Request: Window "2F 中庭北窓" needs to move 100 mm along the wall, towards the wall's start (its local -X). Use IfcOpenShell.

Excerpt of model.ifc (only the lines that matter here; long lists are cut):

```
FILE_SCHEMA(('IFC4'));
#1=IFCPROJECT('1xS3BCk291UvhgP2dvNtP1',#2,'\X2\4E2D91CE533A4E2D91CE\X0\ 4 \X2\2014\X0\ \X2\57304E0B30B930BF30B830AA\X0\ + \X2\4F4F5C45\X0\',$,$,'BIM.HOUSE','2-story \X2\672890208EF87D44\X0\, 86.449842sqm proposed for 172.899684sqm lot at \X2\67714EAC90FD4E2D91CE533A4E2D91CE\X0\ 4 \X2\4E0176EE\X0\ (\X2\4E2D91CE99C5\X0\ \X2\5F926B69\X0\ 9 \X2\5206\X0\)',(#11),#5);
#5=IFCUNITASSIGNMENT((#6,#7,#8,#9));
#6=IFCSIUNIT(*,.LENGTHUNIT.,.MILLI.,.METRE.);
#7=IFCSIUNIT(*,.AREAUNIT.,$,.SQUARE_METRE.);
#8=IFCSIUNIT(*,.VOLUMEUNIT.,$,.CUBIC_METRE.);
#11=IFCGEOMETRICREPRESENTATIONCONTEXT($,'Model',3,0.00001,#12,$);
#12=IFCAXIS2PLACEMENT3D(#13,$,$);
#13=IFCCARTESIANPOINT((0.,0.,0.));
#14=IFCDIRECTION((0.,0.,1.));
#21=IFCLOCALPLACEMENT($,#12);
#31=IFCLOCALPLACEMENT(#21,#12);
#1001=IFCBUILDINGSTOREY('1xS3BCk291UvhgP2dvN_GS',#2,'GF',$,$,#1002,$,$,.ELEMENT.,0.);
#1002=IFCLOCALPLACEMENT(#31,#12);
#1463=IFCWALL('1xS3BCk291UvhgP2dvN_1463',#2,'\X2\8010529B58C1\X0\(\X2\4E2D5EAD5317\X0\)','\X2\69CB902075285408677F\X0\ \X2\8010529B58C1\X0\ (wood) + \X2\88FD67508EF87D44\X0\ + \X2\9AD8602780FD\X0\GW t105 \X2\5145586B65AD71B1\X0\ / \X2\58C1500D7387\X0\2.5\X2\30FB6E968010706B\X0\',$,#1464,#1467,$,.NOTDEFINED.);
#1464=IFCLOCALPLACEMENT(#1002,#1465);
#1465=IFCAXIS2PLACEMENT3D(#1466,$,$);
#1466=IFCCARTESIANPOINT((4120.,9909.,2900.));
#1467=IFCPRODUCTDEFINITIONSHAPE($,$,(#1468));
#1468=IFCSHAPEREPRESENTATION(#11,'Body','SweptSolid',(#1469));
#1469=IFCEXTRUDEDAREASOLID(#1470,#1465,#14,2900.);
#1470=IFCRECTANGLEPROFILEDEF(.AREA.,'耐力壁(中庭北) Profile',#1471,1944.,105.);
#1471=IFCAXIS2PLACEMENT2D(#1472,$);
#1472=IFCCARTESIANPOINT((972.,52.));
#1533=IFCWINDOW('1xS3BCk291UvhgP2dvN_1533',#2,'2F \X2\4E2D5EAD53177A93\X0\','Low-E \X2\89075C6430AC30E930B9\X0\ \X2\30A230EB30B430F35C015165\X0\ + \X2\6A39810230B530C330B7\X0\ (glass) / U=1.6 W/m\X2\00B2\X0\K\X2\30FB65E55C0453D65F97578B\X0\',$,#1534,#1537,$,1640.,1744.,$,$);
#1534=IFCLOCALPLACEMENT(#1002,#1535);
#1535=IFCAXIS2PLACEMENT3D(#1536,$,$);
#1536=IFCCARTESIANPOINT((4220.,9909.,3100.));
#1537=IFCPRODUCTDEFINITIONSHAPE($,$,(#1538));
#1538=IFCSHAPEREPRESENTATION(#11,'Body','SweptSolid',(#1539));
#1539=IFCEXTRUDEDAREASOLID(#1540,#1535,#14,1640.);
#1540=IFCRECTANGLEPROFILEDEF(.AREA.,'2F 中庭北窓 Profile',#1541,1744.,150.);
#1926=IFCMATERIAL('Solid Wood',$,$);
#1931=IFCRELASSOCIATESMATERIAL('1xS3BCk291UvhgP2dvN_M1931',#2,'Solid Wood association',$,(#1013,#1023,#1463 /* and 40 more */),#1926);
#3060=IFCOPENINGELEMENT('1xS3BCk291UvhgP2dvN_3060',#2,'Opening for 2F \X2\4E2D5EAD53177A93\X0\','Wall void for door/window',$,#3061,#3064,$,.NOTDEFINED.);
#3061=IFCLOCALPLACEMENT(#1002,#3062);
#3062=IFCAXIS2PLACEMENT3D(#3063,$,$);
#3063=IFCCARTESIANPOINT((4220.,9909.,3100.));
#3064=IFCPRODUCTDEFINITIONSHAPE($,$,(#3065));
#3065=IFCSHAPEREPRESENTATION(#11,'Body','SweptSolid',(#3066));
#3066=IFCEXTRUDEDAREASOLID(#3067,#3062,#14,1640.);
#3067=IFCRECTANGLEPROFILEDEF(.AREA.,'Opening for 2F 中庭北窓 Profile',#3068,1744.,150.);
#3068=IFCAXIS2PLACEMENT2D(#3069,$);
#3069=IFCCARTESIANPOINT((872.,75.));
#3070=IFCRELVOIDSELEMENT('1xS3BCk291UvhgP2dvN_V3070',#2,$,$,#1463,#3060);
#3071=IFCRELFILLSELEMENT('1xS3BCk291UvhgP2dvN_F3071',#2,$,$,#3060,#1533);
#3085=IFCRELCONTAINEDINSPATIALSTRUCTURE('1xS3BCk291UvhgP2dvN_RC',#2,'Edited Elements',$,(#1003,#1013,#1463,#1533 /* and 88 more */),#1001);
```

```python
import ifcopenshell
import ifcopenshell.api.geometry
import ifcopenshell.util.placement
import ifcopenshell.util.unit

model = ifcopenshell.open("model.ifc")
unit_scale = ifcopenshell.util.unit.calculate_unit_scale(model)

window = model.by_id(1533)
opening = window.FillsVoids[0].RelatingOpeningElement
wall = opening.VoidsElements[0].RelatingBuildingElement

wall_matrix = ifcopenshell.util.placement.get_local_placement(wall.ObjectPlacement)
shift = wall_matrix[:3, 0] * -0.1 / unit_scale
before = ifcopenshell.util.placement.get_local_placement(window.ObjectPlacement)[:3, 3].copy()

# The window is not placed relative to its opening, so move both.
for product in (opening, window):
    matrix = ifcopenshell.util.placement.get_local_placement(product.ObjectPlacement)
    matrix[:3, 3] += shift
    ifcopenshell.api.geometry.edit_object_placement(model, product=product, matrix=matrix, is_si=False)

after = ifcopenshell.util.placement.get_local_placement(window.ObjectPlacement)[:3, 3]
print("window moved by", (after - before).round(3) + 0.0)

model.write("model-out.ifc")
```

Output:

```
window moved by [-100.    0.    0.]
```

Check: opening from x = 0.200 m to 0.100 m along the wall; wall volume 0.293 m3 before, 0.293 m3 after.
